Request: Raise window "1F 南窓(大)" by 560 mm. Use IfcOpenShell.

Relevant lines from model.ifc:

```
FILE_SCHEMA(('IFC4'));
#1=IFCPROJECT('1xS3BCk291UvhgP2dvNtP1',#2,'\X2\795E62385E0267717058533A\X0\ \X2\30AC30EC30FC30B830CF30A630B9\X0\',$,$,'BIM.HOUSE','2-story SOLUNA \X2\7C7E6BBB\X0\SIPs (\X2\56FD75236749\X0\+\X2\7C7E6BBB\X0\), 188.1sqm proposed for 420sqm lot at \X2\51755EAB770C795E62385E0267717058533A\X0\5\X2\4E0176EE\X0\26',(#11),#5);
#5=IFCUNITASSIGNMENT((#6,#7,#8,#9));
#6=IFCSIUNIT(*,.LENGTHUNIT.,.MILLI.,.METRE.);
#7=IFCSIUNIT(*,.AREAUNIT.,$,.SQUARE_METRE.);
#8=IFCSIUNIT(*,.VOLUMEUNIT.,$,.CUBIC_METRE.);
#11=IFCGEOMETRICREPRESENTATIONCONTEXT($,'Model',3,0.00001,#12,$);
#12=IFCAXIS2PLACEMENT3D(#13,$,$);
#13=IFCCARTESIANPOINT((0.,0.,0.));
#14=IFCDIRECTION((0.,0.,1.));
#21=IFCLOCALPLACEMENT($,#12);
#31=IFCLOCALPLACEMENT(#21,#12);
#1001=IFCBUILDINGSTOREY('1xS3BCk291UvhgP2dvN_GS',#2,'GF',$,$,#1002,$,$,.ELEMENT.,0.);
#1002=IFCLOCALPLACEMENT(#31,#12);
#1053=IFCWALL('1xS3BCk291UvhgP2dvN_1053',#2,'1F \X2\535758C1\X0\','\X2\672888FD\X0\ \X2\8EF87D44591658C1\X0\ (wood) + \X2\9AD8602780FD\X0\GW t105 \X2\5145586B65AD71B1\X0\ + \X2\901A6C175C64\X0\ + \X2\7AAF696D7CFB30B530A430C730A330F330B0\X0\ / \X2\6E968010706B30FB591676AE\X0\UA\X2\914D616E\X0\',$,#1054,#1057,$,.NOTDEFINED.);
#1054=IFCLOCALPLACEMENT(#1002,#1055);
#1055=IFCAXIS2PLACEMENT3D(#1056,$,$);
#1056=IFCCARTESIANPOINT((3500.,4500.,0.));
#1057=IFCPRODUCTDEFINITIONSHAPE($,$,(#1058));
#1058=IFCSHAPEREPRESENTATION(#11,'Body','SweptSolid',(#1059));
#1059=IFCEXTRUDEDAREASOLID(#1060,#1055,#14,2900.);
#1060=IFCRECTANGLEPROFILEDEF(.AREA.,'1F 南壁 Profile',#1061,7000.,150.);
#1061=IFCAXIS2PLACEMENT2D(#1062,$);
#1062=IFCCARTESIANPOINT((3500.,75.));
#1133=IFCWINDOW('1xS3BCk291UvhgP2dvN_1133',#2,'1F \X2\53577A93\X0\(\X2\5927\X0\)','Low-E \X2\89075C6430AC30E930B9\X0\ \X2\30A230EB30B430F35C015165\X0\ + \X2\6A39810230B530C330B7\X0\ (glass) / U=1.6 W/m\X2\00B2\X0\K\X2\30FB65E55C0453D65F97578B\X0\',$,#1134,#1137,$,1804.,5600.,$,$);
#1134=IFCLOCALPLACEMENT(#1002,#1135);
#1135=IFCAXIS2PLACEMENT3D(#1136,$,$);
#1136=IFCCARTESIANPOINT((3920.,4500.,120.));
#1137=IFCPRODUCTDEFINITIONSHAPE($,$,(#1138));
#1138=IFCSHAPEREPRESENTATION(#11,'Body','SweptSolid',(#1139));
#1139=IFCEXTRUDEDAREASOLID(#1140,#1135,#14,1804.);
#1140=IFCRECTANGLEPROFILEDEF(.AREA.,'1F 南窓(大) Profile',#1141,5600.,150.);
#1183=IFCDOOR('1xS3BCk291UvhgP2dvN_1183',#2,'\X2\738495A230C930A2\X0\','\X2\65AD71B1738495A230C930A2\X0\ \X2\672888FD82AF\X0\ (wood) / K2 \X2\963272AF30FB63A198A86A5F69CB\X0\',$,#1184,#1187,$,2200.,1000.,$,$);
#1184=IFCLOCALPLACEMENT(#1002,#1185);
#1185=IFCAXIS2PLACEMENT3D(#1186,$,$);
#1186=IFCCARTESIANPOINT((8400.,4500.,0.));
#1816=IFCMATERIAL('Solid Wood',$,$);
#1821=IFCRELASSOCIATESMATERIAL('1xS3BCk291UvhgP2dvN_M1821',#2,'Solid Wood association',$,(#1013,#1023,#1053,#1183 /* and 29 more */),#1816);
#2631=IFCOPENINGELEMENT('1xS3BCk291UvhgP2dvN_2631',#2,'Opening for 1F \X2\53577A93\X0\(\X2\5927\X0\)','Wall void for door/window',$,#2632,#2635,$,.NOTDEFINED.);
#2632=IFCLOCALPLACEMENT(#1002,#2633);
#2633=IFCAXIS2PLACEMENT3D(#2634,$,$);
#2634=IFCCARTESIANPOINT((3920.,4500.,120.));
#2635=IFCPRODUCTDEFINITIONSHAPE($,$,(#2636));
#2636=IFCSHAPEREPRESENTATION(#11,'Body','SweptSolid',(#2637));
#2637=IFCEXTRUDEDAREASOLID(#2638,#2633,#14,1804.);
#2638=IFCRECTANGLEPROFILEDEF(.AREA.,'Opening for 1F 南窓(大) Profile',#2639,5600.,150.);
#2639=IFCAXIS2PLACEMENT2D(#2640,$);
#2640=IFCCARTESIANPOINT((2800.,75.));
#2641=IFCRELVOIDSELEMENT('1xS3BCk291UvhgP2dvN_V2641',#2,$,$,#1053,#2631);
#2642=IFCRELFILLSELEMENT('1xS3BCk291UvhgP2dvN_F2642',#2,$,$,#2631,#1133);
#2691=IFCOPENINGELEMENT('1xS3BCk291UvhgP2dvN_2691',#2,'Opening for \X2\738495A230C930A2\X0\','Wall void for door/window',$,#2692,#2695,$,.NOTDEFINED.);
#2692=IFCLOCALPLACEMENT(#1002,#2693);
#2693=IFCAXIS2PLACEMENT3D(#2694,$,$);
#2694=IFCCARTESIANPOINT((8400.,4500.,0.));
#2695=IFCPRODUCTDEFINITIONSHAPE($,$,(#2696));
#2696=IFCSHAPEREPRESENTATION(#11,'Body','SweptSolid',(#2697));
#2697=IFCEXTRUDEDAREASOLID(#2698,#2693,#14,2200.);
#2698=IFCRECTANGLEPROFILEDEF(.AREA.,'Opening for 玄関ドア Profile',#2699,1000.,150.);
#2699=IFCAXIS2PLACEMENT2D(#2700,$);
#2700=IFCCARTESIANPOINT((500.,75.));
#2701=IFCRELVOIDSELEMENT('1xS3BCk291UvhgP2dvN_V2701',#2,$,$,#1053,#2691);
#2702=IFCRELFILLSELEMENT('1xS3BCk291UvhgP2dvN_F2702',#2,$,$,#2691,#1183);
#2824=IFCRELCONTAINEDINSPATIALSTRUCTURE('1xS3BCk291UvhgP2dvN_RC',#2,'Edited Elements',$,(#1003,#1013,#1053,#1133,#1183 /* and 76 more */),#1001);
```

```python
import numpy as np
import ifcopenshell
import ifcopenshell.api.geometry
import ifcopenshell.util.placement
import ifcopenshell.util.unit

model = ifcopenshell.open("model.ifc")
unit_scale = ifcopenshell.util.unit.calculate_unit_scale(model)

window = model.by_id(1133)
opening = window.FillsVoids[0].RelatingOpeningElement
dz = 0.56 / unit_scale

shift = np.array([0.0, 0.0, dz])
# The window is not placed relative to its opening, so move both.
for product in (opening, window):
    matrix = ifcopenshell.util.placement.get_local_placement(product.ObjectPlacement)
    matrix[:3, 3] += shift
    ifcopenshell.api.geometry.edit_object_placement(model, product=product, matrix=matrix, is_si=False)

print(f"moved by {dz * unit_scale:+.3f} m")

model.write("model_rev.ifc")
```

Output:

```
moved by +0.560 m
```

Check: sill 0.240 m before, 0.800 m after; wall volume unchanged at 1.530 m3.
